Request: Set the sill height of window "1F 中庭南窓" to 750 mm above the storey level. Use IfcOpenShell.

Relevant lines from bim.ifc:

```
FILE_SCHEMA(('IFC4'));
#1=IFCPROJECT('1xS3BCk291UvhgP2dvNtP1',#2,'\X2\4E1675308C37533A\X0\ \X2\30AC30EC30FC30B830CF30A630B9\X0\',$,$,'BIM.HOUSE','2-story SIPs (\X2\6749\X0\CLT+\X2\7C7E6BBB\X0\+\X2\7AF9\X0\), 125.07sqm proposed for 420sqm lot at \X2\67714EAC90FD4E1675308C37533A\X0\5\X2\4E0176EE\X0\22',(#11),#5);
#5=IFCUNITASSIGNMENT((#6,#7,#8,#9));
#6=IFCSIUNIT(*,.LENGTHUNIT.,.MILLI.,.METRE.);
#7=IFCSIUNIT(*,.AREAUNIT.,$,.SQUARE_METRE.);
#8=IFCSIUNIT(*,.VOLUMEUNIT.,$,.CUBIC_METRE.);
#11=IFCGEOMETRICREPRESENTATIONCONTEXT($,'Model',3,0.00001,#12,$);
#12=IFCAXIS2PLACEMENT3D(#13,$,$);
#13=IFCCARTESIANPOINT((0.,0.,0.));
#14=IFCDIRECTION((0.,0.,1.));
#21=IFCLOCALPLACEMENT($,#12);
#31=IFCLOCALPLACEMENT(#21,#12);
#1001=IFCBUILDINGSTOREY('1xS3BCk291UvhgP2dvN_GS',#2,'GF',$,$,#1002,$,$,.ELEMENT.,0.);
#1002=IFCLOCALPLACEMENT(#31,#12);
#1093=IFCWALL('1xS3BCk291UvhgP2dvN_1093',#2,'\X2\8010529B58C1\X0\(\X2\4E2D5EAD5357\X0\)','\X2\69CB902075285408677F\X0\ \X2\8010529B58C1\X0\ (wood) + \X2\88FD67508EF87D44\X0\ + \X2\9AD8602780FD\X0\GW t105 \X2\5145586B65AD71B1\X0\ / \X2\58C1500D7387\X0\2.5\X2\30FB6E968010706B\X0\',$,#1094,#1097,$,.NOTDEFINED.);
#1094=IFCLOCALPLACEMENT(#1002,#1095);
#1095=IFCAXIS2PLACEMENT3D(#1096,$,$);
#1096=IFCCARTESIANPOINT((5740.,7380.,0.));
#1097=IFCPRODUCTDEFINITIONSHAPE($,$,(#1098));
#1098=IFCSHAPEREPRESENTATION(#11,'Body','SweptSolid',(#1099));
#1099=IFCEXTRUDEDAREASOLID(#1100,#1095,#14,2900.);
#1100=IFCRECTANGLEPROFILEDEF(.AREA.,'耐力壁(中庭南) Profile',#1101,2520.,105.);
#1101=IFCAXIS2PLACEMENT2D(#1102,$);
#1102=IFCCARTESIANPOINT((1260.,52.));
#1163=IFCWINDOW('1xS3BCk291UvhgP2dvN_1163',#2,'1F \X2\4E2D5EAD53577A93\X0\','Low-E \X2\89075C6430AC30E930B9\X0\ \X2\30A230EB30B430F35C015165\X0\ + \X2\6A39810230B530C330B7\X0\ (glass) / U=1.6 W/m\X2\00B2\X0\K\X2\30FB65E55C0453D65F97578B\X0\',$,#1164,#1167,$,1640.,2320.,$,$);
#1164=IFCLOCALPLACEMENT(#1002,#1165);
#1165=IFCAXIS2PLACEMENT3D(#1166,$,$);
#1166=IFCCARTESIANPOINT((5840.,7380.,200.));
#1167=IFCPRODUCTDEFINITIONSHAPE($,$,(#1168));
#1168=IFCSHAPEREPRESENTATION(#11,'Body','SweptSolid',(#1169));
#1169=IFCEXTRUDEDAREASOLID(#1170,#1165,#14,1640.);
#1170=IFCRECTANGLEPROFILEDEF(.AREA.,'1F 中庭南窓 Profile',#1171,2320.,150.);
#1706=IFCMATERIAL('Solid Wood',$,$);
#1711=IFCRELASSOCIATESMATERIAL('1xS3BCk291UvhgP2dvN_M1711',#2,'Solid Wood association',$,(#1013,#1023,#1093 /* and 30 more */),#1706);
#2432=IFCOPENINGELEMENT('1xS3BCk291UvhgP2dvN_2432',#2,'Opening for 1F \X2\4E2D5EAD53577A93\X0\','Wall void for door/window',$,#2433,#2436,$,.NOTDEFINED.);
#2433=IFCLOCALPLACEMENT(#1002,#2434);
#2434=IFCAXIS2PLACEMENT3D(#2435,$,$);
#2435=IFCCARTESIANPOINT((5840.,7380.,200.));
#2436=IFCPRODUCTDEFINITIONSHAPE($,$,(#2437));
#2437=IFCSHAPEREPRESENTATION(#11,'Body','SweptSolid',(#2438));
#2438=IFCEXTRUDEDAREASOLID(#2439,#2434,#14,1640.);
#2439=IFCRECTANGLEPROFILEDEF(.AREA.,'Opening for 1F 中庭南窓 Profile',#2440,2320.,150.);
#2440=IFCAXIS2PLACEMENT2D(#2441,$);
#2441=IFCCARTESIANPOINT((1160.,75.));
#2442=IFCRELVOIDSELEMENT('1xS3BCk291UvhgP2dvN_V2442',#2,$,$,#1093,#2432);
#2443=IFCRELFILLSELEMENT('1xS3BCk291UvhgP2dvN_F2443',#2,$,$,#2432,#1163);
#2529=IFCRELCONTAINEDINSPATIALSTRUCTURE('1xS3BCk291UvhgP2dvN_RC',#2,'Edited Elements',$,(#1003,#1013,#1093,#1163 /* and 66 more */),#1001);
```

```python
import numpy as np
import ifcopenshell
import ifcopenshell.api.geometry
import ifcopenshell.geom
import ifcopenshell.util.element
import ifcopenshell.util.placement
import ifcopenshell.util.shape
import ifcopenshell.util.unit

model = ifcopenshell.open("bim.ifc")
unit_scale = ifcopenshell.util.unit.calculate_unit_scale(model)

window = model.by_guid("1xS3BCk291UvhgP2dvN_1163")
opening = window.FillsVoids[0].RelatingOpeningElement
storey = ifcopenshell.util.element.get_container(window, ifc_class="IfcBuildingStorey")
level = ifcopenshell.util.placement.get_local_placement(storey.ObjectPlacement)[2, 3]

# The opening's origin need not be at the sill, so measure its lowest point.
shape = ifcopenshell.geom.create_shape(ifcopenshell.geom.settings(), opening)
bottom = ifcopenshell.util.shape.get_shape_bottom_elevation(shape, shape.geometry) / unit_scale
dz = level + 0.75 / unit_scale - bottom

shift = np.array([0.0, 0.0, dz])
# The window is not placed relative to its opening, so move both.
for product in (opening, window):
    matrix = ifcopenshell.util.placement.get_local_placement(product.ObjectPlacement)
    matrix[:3, 3] += shift
    ifcopenshell.api.geometry.edit_object_placement(model, product=product, matrix=matrix, is_si=False)

print(f"moved by {dz * unit_scale:+.3f} m")

model.write("bim_rev.ifc")
```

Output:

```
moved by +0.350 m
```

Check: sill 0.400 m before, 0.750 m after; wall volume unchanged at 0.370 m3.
